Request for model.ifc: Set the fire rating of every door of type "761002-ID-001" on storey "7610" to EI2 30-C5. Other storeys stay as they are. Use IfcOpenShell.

First a look at what the model holds.

```python
import ifcopenshell
import ifcopenshell.util.element

model = ifcopenshell.open("model.ifc")
print(model.schema)
storey = next(s for s in model.by_type("IfcBuildingStorey") if s.Name == "7610")
doors = [e for e in ifcopenshell.util.element.get_decomposition(storey) if e.is_a("IfcDoor")]
seen = {}
for e in doors:
    element_type = ifcopenshell.util.element.get_type(e)
    key = (element_type.Name if element_type != e and element_type else None, ifcopenshell.util.element.get_pset(e, "Pset_DoorCommon", "FireRating"))
    seen[key] = seen.get(key, 0) + 1
for (name, value), count in sorted(seen.items(), key=str):
    print(count, "x", name, "|", value)
```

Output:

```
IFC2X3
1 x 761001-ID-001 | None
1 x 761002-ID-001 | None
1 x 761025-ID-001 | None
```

```python
import ifcopenshell
import ifcopenshell.api.pset
import ifcopenshell.util.element

model = ifcopenshell.open("model.ifc")

storey = next(s for s in model.by_type("IfcBuildingStorey") if s.Name == "7610")
doors = [e for e in ifcopenshell.util.element.get_decomposition(storey) if e.is_a("IfcDoor")]

count = 0
for e in doors:
    element_type = ifcopenshell.util.element.get_type(e)
    if element_type in (None, e) or element_type.Name != "761002-ID-001":
        continue
    # add_pset returns the element's existing set when there is one.
    pset = ifcopenshell.api.pset.add_pset(model, product=e, name="Pset_DoorCommon")
    ifcopenshell.api.pset.edit_pset(model, pset=pset, properties={"FireRating": "EI2 30-C5"})
    count += 1

print(count, "doors updated")

model.write("model_updated.ifc")
```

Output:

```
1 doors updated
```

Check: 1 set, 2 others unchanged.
